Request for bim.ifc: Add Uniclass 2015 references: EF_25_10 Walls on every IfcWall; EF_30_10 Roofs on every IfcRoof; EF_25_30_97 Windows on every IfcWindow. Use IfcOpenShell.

First a look at what the model holds.

```python
import ifcopenshell

model = ifcopenshell.open("bim.ifc")
print(model.schema)
print("classifications:", [c.Name for c in model.by_type("IfcClassification")])
for ifc_class in ("IfcDoor", "IfcRoof", "IfcStair", "IfcWall", "IfcWindow"):
    print(ifc_class, len(model.by_type(ifc_class)))
```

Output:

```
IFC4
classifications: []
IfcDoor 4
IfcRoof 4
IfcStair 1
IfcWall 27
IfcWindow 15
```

```python
import ifcopenshell
import ifcopenshell.api.classification

model = ifcopenshell.open("bim.ifc")

system = ifcopenshell.api.classification.add_classification(model, classification="Uniclass 2015")

codes = {
    "IfcWall": ("EF_25_10", "Walls"),
    "IfcRoof": ("EF_30_10", "Roofs"),
    "IfcWindow": ("EF_25_30_97", "Windows"),
}
for ifc_class, (code, name) in codes.items():
    products = model.by_type(ifc_class)
    ifcopenshell.api.classification.add_reference(
        model, products=products, classification=system, identification=code, name=name
    )
    print(code, len(products))

model.write("bim_updated.ifc")
```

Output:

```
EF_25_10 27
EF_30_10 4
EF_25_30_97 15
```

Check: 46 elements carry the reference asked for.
